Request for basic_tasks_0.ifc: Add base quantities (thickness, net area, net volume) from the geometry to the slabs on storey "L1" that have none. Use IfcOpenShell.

First a look at what the model holds.

```python
import ifcopenshell
import ifcopenshell.util.element
import ifcopenshell.util.unit

model = ifcopenshell.open("basic_tasks_0.ifc")
print(model.schema)
for unit_type in ("LENGTHUNIT", "AREAUNIT", "VOLUMEUNIT"):
    print(unit_type, ifcopenshell.util.unit.calculate_unit_scale(model, unit_type))
storey = next(s for s in model.by_type("IfcBuildingStorey") if s.Name == "L1")
slabs = [e for e in ifcopenshell.util.element.get_decomposition(storey) if e.is_a("IfcSlab")]
for e in sorted(slabs, key=lambda e: e.id()):
    print(e.id(), e.is_a(), e.Name, list(ifcopenshell.util.element.get_psets(e, qtos_only=True)), sep=" | ")
```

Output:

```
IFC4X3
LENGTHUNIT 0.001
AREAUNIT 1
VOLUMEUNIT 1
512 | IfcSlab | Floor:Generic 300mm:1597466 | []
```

```python
import ifcopenshell
import ifcopenshell.api.pset
import ifcopenshell.geom
import ifcopenshell.util.element
import ifcopenshell.util.shape
import ifcopenshell.util.unit

model = ifcopenshell.open("basic_tasks_0.ifc")
unit_scale = ifcopenshell.util.unit.calculate_unit_scale(model)
area_scale = ifcopenshell.util.unit.calculate_unit_scale(model, "AREAUNIT")
volume_scale = ifcopenshell.util.unit.calculate_unit_scale(model, "VOLUMEUNIT")
settings = ifcopenshell.geom.settings()

storey = next(s for s in model.by_type("IfcBuildingStorey") if s.Name == "L1")
slabs = [e for e in ifcopenshell.util.element.get_decomposition(storey) if e.is_a("IfcSlab")]

for e in sorted(slabs, key=lambda e: e.id()):
    if ifcopenshell.util.element.get_psets(e, qtos_only=True, should_inherit=False):
        continue
    # Geometry comes back in metres, in the element's own axes.
    shape = ifcopenshell.geom.create_shape(settings, e)
    values = {
        "Width": ifcopenshell.util.shape.get_z(shape.geometry) / unit_scale,
        "NetArea": ifcopenshell.util.shape.get_footprint_area(shape.geometry) / area_scale,
        "NetVolume": ifcopenshell.util.shape.get_volume(shape.geometry) / volume_scale,
    }
    qto = ifcopenshell.api.pset.add_qto(model, product=e, name="Qto_SlabBaseQuantities")
    ifcopenshell.api.pset.edit_qto(model, qto=qto, properties=values)
    print(e.id(), {k: round(v, 3) for k, v in values.items()})

model.write("basic_tasks_0_updated.ifc")
```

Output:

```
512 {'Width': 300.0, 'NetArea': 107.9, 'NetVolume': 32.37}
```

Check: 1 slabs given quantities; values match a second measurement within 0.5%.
